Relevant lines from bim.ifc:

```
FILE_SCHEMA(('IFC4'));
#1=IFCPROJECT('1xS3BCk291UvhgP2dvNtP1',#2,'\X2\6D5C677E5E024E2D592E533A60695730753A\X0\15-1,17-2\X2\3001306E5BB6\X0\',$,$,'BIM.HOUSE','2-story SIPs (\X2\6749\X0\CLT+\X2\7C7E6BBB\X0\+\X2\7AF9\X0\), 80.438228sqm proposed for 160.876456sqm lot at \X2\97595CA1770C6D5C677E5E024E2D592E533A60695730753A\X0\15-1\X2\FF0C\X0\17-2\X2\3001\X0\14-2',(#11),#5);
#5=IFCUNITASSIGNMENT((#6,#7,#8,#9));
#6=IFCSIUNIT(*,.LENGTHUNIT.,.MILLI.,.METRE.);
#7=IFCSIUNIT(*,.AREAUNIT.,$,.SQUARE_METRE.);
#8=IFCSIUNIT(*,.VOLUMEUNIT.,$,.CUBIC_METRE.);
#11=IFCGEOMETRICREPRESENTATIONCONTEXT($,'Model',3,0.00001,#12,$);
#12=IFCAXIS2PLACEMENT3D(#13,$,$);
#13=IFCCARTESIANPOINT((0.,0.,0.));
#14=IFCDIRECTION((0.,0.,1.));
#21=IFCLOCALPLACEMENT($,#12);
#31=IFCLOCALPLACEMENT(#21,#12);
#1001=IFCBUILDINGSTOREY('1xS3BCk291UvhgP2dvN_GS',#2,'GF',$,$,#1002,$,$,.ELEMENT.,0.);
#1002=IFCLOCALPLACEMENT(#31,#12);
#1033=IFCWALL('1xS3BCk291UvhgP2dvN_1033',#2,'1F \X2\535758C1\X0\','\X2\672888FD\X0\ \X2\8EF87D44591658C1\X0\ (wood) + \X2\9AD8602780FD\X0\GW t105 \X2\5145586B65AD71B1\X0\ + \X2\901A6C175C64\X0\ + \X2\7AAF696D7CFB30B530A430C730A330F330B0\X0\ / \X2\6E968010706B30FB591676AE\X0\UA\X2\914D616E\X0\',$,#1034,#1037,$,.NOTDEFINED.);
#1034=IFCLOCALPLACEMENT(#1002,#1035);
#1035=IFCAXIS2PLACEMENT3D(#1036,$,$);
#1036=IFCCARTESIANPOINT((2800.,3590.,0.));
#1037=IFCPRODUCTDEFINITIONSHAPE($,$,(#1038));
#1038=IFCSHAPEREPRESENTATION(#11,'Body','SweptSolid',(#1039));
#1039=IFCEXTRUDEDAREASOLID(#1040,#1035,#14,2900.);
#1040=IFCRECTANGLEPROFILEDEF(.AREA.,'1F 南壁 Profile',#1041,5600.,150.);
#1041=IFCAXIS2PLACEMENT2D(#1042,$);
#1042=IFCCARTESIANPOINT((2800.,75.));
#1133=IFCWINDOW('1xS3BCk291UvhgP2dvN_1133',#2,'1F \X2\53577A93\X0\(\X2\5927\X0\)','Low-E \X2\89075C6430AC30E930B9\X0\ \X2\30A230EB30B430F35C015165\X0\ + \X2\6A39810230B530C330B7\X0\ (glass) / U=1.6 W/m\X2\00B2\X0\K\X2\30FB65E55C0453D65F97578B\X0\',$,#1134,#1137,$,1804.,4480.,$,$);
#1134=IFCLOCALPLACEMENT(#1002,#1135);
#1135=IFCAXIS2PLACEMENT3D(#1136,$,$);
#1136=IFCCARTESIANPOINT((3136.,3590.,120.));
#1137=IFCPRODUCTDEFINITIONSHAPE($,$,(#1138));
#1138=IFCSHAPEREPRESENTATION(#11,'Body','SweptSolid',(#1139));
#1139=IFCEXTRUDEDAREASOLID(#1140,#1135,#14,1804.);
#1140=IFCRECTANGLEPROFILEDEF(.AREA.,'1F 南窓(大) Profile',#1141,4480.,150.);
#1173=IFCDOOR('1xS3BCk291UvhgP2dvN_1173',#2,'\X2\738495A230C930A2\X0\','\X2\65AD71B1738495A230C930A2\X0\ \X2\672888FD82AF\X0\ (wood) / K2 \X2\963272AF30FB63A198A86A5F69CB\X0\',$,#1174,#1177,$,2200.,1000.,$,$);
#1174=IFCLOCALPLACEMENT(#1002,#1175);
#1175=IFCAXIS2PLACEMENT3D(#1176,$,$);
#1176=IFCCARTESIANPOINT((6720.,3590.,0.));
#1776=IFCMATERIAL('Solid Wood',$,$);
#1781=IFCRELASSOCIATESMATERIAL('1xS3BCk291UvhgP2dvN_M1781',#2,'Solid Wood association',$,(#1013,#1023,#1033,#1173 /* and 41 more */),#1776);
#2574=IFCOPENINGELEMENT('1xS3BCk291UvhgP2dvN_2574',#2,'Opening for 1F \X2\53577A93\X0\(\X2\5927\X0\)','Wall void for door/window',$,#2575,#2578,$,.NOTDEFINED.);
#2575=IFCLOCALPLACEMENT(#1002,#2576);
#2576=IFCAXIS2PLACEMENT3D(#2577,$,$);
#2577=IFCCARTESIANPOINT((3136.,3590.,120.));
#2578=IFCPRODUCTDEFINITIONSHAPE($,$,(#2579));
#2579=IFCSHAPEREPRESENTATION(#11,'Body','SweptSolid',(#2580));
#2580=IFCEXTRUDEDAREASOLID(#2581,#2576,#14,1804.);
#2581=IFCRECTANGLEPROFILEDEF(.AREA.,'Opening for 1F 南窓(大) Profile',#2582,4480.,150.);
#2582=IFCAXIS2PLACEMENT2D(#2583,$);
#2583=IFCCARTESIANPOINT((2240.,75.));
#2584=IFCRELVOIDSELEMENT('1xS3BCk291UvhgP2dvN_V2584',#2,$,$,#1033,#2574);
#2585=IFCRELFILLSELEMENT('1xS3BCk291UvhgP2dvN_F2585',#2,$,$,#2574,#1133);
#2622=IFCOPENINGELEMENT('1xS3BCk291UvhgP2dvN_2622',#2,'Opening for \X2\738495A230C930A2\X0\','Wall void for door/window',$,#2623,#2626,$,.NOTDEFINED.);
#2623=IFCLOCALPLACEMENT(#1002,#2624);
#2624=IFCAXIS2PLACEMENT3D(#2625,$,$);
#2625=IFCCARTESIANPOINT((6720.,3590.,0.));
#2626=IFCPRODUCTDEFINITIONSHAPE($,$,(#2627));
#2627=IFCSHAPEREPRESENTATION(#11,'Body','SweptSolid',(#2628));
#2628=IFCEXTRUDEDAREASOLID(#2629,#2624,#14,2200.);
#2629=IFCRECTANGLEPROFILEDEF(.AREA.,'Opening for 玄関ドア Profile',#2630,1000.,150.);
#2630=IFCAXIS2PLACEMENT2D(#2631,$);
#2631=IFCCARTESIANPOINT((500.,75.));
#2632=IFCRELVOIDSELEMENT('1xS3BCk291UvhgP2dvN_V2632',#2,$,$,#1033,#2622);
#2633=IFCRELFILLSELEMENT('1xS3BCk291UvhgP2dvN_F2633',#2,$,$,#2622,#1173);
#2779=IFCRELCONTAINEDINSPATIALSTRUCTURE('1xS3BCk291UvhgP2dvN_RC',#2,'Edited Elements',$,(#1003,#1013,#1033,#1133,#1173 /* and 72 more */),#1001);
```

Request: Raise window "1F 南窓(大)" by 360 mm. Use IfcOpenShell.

```python
import numpy as np
import ifcopenshell
import ifcopenshell.api.geometry
import ifcopenshell.util.placement
import ifcopenshell.util.unit

model = ifcopenshell.open("bim.ifc")
unit_scale = ifcopenshell.util.unit.calculate_unit_scale(model)

window = model.by_guid("1xS3BCk291UvhgP2dvN_1133")
opening = window.FillsVoids[0].RelatingOpeningElement
dz = 360.0

shift = np.array([0.0, 0.0, dz])
# The window is not placed relative to its opening, so move both.
for product in (opening, window):
    matrix = ifcopenshell.util.placement.get_local_placement(product.ObjectPlacement)
    matrix[:3, 3] += shift
    ifcopenshell.api.geometry.edit_object_placement(model, product=product, matrix=matrix, is_si=False)

print(f"moved by {dz * unit_scale:+.3f} m")

model.write("bim_updated.ifc")
```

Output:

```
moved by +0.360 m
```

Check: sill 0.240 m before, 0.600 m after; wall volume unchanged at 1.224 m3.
